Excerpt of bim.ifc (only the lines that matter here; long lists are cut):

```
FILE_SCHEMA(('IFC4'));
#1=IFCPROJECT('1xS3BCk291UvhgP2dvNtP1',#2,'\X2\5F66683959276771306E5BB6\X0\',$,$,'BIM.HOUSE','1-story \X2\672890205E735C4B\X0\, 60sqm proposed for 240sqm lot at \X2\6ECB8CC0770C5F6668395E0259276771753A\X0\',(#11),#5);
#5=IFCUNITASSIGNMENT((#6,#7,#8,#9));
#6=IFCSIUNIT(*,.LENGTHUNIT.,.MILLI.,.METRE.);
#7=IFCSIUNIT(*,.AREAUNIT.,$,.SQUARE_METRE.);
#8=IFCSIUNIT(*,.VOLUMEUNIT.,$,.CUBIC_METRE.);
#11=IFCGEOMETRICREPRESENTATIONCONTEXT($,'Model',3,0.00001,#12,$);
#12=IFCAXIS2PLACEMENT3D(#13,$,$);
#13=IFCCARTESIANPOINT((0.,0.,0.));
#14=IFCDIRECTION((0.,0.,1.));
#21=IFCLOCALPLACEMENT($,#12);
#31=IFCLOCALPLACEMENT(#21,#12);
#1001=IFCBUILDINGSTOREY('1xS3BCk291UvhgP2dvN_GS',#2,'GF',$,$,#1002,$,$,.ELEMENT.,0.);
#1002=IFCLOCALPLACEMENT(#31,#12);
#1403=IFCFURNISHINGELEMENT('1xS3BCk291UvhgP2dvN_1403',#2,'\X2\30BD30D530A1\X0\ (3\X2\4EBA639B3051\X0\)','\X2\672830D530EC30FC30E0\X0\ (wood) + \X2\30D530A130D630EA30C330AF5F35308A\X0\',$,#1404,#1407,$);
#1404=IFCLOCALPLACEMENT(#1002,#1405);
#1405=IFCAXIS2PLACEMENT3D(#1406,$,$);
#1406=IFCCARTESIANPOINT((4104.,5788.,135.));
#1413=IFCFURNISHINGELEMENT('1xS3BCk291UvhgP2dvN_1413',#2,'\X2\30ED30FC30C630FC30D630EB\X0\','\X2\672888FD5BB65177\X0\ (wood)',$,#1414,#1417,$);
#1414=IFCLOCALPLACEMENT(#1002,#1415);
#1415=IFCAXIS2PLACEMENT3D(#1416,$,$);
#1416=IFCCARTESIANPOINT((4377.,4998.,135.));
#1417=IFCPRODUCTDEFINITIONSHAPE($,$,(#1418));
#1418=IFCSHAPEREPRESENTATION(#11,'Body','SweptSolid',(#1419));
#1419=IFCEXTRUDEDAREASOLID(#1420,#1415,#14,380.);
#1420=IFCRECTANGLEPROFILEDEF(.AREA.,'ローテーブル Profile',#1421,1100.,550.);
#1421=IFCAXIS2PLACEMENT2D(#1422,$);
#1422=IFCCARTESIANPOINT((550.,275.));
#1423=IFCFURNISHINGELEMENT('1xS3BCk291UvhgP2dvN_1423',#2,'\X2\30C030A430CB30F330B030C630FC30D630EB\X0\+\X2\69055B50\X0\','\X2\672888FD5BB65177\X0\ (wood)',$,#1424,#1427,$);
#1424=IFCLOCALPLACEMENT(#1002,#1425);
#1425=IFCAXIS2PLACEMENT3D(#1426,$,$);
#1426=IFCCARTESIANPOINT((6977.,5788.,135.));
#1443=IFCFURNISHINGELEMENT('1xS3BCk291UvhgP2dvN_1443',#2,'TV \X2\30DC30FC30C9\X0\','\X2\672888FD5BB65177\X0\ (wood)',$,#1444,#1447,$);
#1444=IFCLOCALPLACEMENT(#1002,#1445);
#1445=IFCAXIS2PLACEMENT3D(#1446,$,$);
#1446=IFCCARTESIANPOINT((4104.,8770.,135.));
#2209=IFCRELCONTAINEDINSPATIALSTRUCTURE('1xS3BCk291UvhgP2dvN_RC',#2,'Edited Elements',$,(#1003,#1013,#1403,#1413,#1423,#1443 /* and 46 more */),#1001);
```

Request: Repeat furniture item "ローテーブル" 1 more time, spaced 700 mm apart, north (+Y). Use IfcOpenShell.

```python
import numpy as np
import ifcopenshell
import ifcopenshell.api.geometry
import ifcopenshell.api.root
import ifcopenshell.util.element
import ifcopenshell.util.placement
import ifcopenshell.util.unit

model = ifcopenshell.open("bim.ifc")
unit_scale = ifcopenshell.util.unit.calculate_unit_scale(model)


def reuse_history(source, copy):
    """copy_class also copies each property set's owner history, people and application; keep the originals."""
    for rel in copy.IsDefinedBy:
        if rel.is_a("IfcRelDefinesByProperties") and (history := rel.RelatingPropertyDefinition.OwnerHistory):
            rel.RelatingPropertyDefinition.OwnerHistory = source.OwnerHistory
            ifcopenshell.util.element.remove_deep2(model, history)


source = model.by_guid("1xS3BCk291UvhgP2dvN_1413")
base = ifcopenshell.util.placement.get_local_placement(source.ObjectPlacement)
step = np.array([0.0, 1.0, 0.0]) * 0.7 / unit_scale

for i in range(1, 2):
    copy = ifcopenshell.api.root.copy_class(model, product=source)
    copy.Representation = ifcopenshell.util.element.copy_deep(
        model, source.Representation, exclude=["IfcGeometricRepresentationContext", "IfcRepresentationMap"]
    )
    reuse_history(source, copy)
    matrix = base.copy()
    matrix[:3, 3] += i * step
    print("added at", matrix[:3, 3].round(3) + 0.0)
    ifcopenshell.api.geometry.edit_object_placement(model, product=copy, matrix=matrix, is_si=False)

model.write("bim_edited.ifc")
```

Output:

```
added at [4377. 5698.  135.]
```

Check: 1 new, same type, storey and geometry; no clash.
